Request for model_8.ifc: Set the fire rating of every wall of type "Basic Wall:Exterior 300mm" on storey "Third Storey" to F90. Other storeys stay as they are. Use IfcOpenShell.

First a look at what the model holds.

```python
import ifcopenshell
import ifcopenshell.util.element

model = ifcopenshell.open("model_8.ifc")
print(model.schema)
storey = next(s for s in model.by_type("IfcBuildingStorey") if s.Name == "Third Storey")
walls = [e for e in ifcopenshell.util.element.get_decomposition(storey) if e.is_a("IfcWall")]
seen = {}
for e in walls:
    element_type = ifcopenshell.util.element.get_type(e)
    key = (element_type.Name if element_type != e and element_type else None, ifcopenshell.util.element.get_pset(e, "Pset_WallCommon", "FireRating"))
    seen[key] = seen.get(key, 0) + 1
for (name, value), count in sorted(seen.items(), key=str):
    print(count, "x", name, "|", value)
```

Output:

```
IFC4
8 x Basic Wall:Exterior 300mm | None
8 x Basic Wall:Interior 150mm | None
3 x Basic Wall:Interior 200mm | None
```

```python
import ifcopenshell
import ifcopenshell.api.pset
import ifcopenshell.util.element

model = ifcopenshell.open("model_8.ifc")

storey = next(s for s in model.by_type("IfcBuildingStorey") if s.Name == "Third Storey")
walls = [e for e in ifcopenshell.util.element.get_decomposition(storey) if e.is_a("IfcWall")]

count = 0
for e in walls:
    element_type = ifcopenshell.util.element.get_type(e)
    if element_type in (None, e) or element_type.Name != "Basic Wall:Exterior 300mm":
        continue
    # add_pset returns the element's existing set when there is one.
    pset = ifcopenshell.api.pset.add_pset(model, product=e, name="Pset_WallCommon")
    ifcopenshell.api.pset.edit_pset(model, pset=pset, properties={"FireRating": "F90"})
    count += 1

print(count, "walls updated")

model.write("model_8_rev.ifc")
```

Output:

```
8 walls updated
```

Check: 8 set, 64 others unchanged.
